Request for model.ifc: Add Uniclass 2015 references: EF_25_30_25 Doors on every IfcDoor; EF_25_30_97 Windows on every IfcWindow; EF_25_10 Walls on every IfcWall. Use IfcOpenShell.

First a look at what the model holds.

```python
import ifcopenshell

model = ifcopenshell.open("model.ifc")
print(model.schema)
print("classifications:", [c.Name for c in model.by_type("IfcClassification")])
for ifc_class in ("IfcDoor", "IfcRoof", "IfcStair", "IfcWall", "IfcWindow"):
    print(ifc_class, len(model.by_type(ifc_class)))
```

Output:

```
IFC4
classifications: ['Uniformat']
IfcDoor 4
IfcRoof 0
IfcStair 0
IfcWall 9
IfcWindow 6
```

```python
import ifcopenshell
import ifcopenshell.api.classification

model = ifcopenshell.open("model.ifc")

system = ifcopenshell.api.classification.add_classification(model, classification="Uniclass 2015")

codes = {
    "IfcDoor": ("EF_25_30_25", "Doors"),
    "IfcWindow": ("EF_25_30_97", "Windows"),
    "IfcWall": ("EF_25_10", "Walls"),
}
for ifc_class, (code, name) in codes.items():
    products = model.by_type(ifc_class)
    ifcopenshell.api.classification.add_reference(
        model, products=products, classification=system, identification=code, name=name
    )
    print(code, len(products))

model.write("model_updated.ifc")
```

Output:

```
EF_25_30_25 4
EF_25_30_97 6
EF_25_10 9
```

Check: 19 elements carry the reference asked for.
